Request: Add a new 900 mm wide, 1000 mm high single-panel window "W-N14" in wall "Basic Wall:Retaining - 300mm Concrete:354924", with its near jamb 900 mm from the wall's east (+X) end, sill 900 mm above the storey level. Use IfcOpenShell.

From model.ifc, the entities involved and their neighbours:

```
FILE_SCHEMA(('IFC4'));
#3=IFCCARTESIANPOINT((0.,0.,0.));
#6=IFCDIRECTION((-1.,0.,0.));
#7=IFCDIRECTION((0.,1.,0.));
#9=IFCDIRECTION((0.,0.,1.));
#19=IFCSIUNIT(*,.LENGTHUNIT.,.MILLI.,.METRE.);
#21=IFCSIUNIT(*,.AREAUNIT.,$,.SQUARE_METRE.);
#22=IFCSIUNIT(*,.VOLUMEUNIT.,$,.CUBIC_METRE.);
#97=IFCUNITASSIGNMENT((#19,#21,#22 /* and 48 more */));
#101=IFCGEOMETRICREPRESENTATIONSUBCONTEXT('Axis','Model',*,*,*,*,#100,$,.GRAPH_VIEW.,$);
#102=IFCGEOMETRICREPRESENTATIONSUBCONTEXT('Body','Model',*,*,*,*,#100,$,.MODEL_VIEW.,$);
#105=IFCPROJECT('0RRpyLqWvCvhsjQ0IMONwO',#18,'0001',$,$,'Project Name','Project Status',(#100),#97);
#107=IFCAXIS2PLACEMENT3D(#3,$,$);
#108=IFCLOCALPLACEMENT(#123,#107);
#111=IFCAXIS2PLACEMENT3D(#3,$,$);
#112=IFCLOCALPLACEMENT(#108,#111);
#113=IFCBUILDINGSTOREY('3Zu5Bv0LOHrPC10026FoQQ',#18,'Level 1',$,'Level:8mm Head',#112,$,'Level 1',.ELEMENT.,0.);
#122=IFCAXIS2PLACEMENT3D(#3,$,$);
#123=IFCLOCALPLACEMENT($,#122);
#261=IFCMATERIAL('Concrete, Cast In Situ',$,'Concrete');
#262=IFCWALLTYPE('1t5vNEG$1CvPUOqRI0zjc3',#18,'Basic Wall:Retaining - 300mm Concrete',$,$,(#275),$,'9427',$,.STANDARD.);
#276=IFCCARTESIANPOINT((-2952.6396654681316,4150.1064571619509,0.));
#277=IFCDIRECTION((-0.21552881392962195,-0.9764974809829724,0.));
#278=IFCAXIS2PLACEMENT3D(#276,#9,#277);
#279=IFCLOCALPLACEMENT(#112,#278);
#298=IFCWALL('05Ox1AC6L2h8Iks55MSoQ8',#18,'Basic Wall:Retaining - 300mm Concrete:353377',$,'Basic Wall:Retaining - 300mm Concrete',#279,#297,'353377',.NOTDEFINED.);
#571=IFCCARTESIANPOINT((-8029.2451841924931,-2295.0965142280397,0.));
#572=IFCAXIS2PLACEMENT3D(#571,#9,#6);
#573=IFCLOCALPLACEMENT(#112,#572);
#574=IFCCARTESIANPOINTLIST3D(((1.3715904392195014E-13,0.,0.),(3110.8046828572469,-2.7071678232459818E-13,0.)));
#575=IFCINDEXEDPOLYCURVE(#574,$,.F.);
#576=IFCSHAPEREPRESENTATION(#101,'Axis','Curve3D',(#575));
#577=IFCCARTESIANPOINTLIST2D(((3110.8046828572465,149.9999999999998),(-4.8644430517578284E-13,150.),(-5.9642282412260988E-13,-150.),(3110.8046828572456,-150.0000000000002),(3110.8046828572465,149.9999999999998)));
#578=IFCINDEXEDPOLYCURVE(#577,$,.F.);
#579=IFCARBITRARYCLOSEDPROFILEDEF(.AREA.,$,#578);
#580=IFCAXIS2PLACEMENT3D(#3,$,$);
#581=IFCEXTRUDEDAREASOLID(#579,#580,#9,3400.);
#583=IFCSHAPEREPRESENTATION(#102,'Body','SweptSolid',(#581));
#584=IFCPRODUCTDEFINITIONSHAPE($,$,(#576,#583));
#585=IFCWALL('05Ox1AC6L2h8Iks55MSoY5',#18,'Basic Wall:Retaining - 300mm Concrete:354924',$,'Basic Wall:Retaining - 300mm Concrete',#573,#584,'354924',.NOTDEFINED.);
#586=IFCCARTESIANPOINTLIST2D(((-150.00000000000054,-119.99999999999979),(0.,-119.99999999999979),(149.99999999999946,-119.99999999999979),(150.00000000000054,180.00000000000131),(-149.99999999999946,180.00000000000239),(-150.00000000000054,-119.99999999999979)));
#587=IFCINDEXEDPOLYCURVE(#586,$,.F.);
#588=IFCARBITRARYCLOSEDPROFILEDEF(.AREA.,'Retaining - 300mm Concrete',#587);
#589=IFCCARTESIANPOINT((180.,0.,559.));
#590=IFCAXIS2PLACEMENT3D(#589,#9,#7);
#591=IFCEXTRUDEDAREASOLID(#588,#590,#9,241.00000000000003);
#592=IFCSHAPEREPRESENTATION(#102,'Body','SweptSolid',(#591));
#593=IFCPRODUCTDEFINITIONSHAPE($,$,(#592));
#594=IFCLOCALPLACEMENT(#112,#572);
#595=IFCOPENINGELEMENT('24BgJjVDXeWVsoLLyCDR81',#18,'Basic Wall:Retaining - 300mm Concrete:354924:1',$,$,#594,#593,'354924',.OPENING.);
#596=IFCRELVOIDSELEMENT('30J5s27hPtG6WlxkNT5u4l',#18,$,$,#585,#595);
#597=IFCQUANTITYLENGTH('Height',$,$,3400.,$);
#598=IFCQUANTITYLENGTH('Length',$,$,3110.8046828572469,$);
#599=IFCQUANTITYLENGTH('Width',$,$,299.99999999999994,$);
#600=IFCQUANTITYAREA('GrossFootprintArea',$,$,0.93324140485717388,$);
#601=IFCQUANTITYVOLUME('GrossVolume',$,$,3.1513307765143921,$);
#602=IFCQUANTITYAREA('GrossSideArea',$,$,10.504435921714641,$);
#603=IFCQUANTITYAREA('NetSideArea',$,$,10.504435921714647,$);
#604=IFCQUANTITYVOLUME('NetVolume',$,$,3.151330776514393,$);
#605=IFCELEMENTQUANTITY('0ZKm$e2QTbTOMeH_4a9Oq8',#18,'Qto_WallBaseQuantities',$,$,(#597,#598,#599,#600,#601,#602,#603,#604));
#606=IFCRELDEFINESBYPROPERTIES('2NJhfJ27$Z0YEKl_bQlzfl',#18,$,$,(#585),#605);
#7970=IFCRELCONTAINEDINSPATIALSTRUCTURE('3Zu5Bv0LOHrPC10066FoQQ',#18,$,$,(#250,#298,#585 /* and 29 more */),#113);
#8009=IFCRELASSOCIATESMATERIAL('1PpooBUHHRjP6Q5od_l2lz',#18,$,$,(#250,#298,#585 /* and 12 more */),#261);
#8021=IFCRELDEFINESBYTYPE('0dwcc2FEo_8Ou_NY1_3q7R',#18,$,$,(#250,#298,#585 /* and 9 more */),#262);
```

```python
import numpy as np
import ifcopenshell
import ifcopenshell.api.feature
import ifcopenshell.api.geometry
import ifcopenshell.api.pset
import ifcopenshell.api.root
import ifcopenshell.api.spatial
import ifcopenshell.geom
import ifcopenshell.util.element
import ifcopenshell.util.placement
import ifcopenshell.util.representation
import ifcopenshell.util.shape
import ifcopenshell.util.unit

model = ifcopenshell.open("model.ifc")
unit_scale = ifcopenshell.util.unit.calculate_unit_scale(model)
area_scale = ifcopenshell.util.unit.calculate_unit_scale(model, "AREAUNIT")
volume_scale = ifcopenshell.util.unit.calculate_unit_scale(model, "VOLUMEUNIT")
settings = ifcopenshell.geom.settings()


def volume(element):
    """Net volume in cubic metres, openings subtracted."""
    shape = ifcopenshell.geom.create_shape(settings, element)
    return ifcopenshell.util.shape.get_volume(shape.geometry)


wall = model.by_guid("05Ox1AC6L2h8Iks55MSoY5")
storey = ifcopenshell.util.element.get_container(wall, ifc_class="IfcBuildingStorey")
context = ifcopenshell.util.representation.get_context(model, "Model", "Body", "MODEL_VIEW")
before = volume(wall)

width, height, from_end, sill = 0.9, 1, 0.9, 0.9  # metres

# The wall runs along its own X axis, and the end named is its -X end.
wall_shape = ifcopenshell.geom.create_shape(settings, wall)
x, y, z = ifcopenshell.util.shape.get_vertices(wall_shape.geometry).T
start = x.min() + from_end
face, thickness = float(y.min()), float(y.max() - y.min())
wall_matrix = ifcopenshell.util.placement.get_local_placement(wall.ObjectPlacement)
level = ifcopenshell.util.placement.get_local_placement(storey.ObjectPlacement)[2, 3]


def in_wall(x, y):
    """Placement at x, y metres in the wall's axes, at sill height."""
    matrix = wall_matrix.copy()
    matrix[:, 3] = wall_matrix @ np.array([x / unit_scale, y / unit_scale, 0.0, 1.0])
    matrix[2, 3] = level + sill / unit_scale
    return matrix


# Opening: a box that overshoots both wall faces by 50 mm.
opening = ifcopenshell.api.root.create_entity(model, ifc_class="IfcOpeningElement", predefined_type="OPENING")
box = ifcopenshell.api.geometry.add_wall_representation(
    model, context=context, length=width, height=height, thickness=thickness + 0.1
)
ifcopenshell.api.geometry.assign_representation(model, product=opening, representation=box)
ifcopenshell.api.geometry.edit_object_placement(model, product=opening, matrix=in_wall(start, face - 0.05), is_si=False)
ifcopenshell.api.feature.add_feature(model, feature=opening, element=wall)

window = ifcopenshell.api.root.create_entity(model, ifc_class="IfcWindow", name="W-N14", predefined_type="WINDOW")
window.OverallWidth, window.OverallHeight = width / unit_scale, height / unit_scale
window.PartitioningType = "SINGLE_PANEL"
body = ifcopenshell.api.geometry.add_window_representation(
    model,
    context=context,
    overall_width=window.OverallWidth,
    overall_height=window.OverallHeight,
    partition_type="SINGLE_PANEL",
)
ifcopenshell.api.geometry.assign_representation(model, product=window, representation=body)
ifcopenshell.api.spatial.assign_container(model, products=[window], relating_structure=storey)
ifcopenshell.api.feature.add_filling(model, opening=opening, element=window)

# Centre the window in the wall's thickness.
ifcopenshell.api.geometry.edit_object_placement(model, product=window, matrix=in_wall(start, face), is_si=False)
window_shape = ifcopenshell.geom.create_shape(settings, window)
depth = ifcopenshell.util.shape.get_vertices(window_shape.geometry)[:, 1]
offset = face + thickness / 2 - (depth.min() + depth.max()) / 2
ifcopenshell.api.geometry.edit_object_placement(model, product=window, matrix=in_wall(start, offset), is_si=False)

after = volume(wall)

# Update the wall's stored quantities.
qto = model.by_id(ifcopenshell.util.element.get_pset(wall, "Qto_WallBaseQuantities", should_inherit=False)["id"])
ifcopenshell.api.pset.edit_qto(model, qto=qto, properties={
    "NetSideArea": after / thickness / area_scale,
    "NetVolume": after / volume_scale,
})

print(f"wall volume {before:.3f} -> {after:.3f} m3")

model.write("model_v2.ifc")
```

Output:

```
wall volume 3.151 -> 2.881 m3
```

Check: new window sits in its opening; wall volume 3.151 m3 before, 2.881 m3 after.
